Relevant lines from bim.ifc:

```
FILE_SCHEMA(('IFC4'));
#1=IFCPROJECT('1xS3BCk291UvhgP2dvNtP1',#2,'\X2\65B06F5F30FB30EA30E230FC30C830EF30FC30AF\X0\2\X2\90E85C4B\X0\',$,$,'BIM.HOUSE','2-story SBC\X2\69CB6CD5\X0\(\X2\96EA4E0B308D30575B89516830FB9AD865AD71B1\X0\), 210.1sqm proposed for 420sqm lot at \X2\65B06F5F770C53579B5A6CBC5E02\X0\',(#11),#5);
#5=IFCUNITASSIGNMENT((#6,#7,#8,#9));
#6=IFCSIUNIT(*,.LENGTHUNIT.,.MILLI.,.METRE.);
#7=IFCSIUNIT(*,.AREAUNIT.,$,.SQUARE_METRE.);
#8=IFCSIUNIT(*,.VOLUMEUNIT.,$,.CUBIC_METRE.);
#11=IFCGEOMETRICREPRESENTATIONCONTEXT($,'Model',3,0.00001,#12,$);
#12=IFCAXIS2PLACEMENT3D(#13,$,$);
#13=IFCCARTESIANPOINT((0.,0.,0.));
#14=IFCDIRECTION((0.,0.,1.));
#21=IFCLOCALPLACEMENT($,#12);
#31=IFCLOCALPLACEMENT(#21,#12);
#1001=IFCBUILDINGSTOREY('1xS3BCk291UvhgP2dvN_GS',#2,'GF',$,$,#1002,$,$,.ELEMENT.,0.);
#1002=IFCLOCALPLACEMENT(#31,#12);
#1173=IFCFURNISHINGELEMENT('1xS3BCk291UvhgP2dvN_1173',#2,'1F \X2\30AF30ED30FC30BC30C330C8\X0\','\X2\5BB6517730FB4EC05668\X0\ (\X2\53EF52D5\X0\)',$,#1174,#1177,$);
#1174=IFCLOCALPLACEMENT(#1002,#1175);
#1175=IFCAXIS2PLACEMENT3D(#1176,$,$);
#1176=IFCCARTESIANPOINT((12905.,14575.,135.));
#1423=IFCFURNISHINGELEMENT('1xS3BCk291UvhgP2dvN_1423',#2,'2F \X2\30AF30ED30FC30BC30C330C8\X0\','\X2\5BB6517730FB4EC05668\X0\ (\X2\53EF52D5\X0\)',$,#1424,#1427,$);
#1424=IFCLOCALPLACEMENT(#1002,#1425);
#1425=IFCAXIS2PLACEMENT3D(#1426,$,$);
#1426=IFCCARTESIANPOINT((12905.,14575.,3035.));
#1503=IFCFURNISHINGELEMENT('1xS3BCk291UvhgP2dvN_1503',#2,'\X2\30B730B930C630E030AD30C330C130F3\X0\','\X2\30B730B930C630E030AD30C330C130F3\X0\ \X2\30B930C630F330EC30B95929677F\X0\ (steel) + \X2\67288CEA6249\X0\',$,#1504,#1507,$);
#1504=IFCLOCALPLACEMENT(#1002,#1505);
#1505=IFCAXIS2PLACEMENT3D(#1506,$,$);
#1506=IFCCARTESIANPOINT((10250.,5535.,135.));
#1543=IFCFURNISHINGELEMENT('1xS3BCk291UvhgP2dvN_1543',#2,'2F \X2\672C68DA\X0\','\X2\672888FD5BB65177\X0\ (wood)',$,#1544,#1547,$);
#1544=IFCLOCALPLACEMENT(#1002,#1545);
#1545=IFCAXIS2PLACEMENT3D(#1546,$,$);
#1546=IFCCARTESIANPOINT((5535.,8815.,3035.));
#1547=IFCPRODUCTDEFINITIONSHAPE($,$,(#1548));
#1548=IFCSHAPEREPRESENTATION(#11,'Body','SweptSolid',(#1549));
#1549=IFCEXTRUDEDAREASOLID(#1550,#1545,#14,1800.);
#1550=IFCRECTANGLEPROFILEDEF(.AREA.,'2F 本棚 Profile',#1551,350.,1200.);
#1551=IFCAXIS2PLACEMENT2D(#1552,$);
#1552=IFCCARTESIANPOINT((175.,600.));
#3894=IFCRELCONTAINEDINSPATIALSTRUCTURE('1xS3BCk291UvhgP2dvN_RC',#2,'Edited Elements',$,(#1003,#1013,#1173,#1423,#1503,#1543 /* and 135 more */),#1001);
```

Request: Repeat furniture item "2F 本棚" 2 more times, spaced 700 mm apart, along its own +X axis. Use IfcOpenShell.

```python
import ifcopenshell
import ifcopenshell.api.geometry
import ifcopenshell.api.root
import ifcopenshell.util.element
import ifcopenshell.util.placement
import ifcopenshell.util.unit

model = ifcopenshell.open("bim.ifc")
unit_scale = ifcopenshell.util.unit.calculate_unit_scale(model)


def reuse_history(source, copy):
    """copy_class also copies each property set's owner history, people and application; keep the originals."""
    for rel in copy.IsDefinedBy:
        if rel.is_a("IfcRelDefinesByProperties") and (history := rel.RelatingPropertyDefinition.OwnerHistory):
            rel.RelatingPropertyDefinition.OwnerHistory = source.OwnerHistory
            ifcopenshell.util.element.remove_deep2(model, history)


source = model.by_guid("1xS3BCk291UvhgP2dvN_1543")
base = ifcopenshell.util.placement.get_local_placement(source.ObjectPlacement)
step = base[:3, 0] * 0.7 / unit_scale

for i in range(1, 3):
    copy = ifcopenshell.api.root.copy_class(model, product=source)
    copy.Representation = ifcopenshell.util.element.copy_deep(
        model, source.Representation, exclude=["IfcGeometricRepresentationContext", "IfcRepresentationMap"]
    )
    reuse_history(source, copy)
    matrix = base.copy()
    matrix[:3, 3] += i * step
    print("added at", matrix[:3, 3].round(3) + 0.0)
    ifcopenshell.api.geometry.edit_object_placement(model, product=copy, matrix=matrix, is_si=False)

model.write("bim-out.ifc")
```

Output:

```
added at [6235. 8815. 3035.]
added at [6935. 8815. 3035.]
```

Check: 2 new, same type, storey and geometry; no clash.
